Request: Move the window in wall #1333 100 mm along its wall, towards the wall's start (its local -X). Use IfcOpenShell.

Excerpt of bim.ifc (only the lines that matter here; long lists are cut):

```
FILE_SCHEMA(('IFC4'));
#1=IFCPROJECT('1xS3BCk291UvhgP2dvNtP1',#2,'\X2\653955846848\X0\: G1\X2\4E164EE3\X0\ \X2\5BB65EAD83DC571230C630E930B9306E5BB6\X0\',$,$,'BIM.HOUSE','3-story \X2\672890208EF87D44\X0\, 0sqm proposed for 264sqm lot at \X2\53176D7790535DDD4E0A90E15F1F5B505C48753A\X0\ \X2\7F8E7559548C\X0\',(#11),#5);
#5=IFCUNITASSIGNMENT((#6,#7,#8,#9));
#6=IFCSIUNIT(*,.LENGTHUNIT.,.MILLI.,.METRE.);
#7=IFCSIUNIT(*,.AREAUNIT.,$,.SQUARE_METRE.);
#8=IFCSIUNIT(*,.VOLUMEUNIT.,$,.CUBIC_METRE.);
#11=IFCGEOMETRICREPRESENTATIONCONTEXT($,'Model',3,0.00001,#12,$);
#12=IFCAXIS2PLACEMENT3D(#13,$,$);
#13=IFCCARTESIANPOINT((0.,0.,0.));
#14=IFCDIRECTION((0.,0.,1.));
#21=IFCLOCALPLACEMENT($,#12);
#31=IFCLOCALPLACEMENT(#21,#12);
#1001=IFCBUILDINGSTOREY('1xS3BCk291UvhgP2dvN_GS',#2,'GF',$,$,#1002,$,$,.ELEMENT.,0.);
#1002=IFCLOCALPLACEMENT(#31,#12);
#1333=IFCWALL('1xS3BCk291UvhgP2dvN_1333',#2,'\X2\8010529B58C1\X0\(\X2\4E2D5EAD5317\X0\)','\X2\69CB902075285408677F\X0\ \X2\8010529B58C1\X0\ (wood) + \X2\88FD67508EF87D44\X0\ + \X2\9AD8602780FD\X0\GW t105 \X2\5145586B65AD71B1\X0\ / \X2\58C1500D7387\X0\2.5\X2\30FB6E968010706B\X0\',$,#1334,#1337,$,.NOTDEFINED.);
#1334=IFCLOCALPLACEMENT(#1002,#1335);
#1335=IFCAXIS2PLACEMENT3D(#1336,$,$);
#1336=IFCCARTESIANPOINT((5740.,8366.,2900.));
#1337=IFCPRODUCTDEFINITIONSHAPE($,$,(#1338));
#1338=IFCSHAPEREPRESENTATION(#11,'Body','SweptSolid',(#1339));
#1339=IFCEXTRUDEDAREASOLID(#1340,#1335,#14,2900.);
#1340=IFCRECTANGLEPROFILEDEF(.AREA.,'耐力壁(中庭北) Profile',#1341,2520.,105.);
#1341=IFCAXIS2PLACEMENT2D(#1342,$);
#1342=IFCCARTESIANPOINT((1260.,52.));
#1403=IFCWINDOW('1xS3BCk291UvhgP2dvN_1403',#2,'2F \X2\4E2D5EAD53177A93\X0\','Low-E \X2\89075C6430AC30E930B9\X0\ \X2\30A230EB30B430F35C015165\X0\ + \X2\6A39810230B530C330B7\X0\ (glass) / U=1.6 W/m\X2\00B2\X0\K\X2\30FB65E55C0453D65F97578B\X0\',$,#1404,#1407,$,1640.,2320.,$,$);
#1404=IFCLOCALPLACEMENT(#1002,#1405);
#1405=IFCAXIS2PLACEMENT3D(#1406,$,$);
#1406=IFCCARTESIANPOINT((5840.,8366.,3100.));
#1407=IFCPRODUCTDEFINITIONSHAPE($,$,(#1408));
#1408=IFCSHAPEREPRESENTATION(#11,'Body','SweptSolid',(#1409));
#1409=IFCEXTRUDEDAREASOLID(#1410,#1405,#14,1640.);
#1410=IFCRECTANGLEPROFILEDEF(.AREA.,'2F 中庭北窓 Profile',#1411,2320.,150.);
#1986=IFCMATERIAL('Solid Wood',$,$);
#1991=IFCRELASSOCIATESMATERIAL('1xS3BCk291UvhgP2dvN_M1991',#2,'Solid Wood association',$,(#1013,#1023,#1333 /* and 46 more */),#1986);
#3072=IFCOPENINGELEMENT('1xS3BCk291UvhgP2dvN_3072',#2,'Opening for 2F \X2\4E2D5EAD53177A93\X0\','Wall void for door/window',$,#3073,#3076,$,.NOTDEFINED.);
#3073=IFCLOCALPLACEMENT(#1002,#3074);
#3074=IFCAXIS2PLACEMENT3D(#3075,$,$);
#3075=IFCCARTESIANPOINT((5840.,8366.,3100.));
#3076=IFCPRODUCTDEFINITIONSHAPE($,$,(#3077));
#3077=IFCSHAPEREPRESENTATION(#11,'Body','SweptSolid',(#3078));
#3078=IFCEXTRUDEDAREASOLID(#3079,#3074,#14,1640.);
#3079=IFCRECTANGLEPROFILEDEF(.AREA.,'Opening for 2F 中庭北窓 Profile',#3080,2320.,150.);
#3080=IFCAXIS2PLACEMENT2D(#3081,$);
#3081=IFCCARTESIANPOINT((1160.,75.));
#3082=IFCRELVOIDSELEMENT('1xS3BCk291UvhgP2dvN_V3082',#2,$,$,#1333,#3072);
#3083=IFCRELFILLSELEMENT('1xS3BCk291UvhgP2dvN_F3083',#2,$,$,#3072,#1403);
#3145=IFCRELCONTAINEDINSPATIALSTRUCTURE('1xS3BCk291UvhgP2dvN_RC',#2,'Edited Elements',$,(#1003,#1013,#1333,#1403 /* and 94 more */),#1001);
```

```python
import ifcopenshell
import ifcopenshell.api.geometry
import ifcopenshell.util.placement
import ifcopenshell.util.unit

model = ifcopenshell.open("bim.ifc")
unit_scale = ifcopenshell.util.unit.calculate_unit_scale(model)

window = model.by_guid("1xS3BCk291UvhgP2dvN_1403")
opening = window.FillsVoids[0].RelatingOpeningElement
wall = opening.VoidsElements[0].RelatingBuildingElement

wall_matrix = ifcopenshell.util.placement.get_local_placement(wall.ObjectPlacement)
shift = wall_matrix[:3, 0] * -0.1 / unit_scale
before = ifcopenshell.util.placement.get_local_placement(window.ObjectPlacement)[:3, 3].copy()

# The window is not placed relative to its opening, so move both.
for product in (opening, window):
    matrix = ifcopenshell.util.placement.get_local_placement(product.ObjectPlacement)
    matrix[:3, 3] += shift
    ifcopenshell.api.geometry.edit_object_placement(model, product=product, matrix=matrix, is_si=False)

after = ifcopenshell.util.placement.get_local_placement(window.ObjectPlacement)[:3, 3]
print("window moved by", (after - before).round(3) + 0.0)

model.write("bim_updated.ifc")
```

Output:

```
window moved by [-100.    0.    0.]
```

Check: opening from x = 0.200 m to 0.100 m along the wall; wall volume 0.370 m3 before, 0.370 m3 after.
